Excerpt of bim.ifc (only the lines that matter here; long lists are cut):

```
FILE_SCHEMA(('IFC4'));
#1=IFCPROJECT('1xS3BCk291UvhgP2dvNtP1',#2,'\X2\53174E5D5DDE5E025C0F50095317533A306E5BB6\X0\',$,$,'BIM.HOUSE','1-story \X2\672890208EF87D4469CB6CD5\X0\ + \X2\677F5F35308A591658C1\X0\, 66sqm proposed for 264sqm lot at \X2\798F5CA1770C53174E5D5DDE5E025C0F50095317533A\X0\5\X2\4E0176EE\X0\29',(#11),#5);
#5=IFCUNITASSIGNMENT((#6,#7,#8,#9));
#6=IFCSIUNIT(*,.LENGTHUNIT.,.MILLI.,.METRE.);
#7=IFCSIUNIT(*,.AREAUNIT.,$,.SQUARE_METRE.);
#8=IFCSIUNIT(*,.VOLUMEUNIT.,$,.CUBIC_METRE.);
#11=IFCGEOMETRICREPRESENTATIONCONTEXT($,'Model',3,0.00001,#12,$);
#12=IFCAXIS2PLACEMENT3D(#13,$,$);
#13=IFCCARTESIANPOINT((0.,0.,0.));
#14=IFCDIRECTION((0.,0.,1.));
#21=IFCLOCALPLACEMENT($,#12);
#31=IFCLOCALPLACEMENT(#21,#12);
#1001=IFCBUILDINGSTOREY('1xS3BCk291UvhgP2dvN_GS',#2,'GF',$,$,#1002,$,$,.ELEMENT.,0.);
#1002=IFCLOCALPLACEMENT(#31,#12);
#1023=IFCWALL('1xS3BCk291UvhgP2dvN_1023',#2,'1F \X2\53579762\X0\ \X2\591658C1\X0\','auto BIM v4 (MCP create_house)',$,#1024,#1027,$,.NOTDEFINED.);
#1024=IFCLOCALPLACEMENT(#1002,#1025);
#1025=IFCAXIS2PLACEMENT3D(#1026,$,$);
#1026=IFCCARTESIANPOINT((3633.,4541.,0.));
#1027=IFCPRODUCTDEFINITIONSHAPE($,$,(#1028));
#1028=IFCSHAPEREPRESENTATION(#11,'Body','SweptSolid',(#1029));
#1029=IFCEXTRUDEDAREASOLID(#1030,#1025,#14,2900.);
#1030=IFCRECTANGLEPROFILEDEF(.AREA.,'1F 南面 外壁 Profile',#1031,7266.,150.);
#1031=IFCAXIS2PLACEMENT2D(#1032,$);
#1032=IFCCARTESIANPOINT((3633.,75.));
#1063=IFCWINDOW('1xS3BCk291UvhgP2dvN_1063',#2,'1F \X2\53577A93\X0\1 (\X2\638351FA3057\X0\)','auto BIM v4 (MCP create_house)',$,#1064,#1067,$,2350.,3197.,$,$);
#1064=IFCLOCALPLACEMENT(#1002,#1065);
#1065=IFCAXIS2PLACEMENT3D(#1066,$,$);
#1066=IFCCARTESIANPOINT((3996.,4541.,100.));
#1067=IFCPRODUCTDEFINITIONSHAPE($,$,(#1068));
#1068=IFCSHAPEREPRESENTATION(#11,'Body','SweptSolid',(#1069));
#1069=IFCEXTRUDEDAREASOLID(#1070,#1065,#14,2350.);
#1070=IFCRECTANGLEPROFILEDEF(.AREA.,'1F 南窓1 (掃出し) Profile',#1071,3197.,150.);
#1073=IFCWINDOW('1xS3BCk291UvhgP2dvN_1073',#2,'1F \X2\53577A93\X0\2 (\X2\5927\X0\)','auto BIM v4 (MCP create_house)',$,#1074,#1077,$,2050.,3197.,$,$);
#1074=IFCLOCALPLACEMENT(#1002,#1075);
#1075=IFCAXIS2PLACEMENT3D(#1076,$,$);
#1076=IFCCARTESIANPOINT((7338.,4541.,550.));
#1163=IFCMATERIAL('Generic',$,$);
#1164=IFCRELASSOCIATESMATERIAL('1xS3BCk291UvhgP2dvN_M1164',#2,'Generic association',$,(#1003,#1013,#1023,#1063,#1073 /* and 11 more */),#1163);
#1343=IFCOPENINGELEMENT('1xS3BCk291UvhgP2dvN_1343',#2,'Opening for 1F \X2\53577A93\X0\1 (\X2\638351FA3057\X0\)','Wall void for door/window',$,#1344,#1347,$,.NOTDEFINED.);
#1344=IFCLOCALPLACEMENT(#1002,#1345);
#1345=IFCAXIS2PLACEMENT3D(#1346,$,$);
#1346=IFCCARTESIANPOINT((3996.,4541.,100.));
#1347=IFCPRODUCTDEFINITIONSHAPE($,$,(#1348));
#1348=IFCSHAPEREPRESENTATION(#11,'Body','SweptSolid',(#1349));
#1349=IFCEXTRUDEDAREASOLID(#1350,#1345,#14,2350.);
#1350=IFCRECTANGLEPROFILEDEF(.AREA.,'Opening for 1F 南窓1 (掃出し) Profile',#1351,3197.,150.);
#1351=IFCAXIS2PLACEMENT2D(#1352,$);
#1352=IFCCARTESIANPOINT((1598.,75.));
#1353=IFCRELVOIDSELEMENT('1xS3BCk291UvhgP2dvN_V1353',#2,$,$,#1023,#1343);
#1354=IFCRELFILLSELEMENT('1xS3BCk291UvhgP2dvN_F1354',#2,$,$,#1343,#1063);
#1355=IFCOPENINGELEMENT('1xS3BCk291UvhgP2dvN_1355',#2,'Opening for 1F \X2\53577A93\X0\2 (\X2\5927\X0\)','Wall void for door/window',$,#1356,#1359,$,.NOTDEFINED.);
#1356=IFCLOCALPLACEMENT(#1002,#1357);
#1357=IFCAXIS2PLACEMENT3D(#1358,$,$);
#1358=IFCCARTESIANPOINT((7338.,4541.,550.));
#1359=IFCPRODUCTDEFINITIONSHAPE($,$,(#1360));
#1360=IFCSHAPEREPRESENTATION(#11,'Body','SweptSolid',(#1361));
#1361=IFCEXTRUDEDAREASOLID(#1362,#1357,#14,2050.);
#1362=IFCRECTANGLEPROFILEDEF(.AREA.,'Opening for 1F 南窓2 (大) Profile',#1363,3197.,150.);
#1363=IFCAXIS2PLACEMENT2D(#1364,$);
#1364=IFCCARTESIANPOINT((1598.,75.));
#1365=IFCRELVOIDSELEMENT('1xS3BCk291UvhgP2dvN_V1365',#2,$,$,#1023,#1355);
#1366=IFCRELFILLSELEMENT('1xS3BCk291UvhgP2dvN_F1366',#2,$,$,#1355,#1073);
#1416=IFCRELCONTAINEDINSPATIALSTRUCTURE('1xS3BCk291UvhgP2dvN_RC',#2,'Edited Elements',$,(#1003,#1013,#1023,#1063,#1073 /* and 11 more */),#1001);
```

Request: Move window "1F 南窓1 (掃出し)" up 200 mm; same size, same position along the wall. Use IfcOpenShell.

```python
import numpy as np
import ifcopenshell
import ifcopenshell.api.geometry
import ifcopenshell.util.placement
import ifcopenshell.util.unit

model = ifcopenshell.open("bim.ifc")
unit_scale = ifcopenshell.util.unit.calculate_unit_scale(model)

window = model.by_guid("1xS3BCk291UvhgP2dvN_1063")
opening = window.FillsVoids[0].RelatingOpeningElement
dz = 0.2 / unit_scale

shift = np.array([0.0, 0.0, dz])
# The window is not placed relative to its opening, so move both.
for product in (opening, window):
    matrix = ifcopenshell.util.placement.get_local_placement(product.ObjectPlacement)
    matrix[:3, 3] += shift
    ifcopenshell.api.geometry.edit_object_placement(model, product=product, matrix=matrix, is_si=False)

print(f"moved by {dz * unit_scale:+.3f} m")

model.write("bim_rev.ifc")
```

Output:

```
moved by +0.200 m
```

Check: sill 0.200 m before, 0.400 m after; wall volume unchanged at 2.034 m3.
